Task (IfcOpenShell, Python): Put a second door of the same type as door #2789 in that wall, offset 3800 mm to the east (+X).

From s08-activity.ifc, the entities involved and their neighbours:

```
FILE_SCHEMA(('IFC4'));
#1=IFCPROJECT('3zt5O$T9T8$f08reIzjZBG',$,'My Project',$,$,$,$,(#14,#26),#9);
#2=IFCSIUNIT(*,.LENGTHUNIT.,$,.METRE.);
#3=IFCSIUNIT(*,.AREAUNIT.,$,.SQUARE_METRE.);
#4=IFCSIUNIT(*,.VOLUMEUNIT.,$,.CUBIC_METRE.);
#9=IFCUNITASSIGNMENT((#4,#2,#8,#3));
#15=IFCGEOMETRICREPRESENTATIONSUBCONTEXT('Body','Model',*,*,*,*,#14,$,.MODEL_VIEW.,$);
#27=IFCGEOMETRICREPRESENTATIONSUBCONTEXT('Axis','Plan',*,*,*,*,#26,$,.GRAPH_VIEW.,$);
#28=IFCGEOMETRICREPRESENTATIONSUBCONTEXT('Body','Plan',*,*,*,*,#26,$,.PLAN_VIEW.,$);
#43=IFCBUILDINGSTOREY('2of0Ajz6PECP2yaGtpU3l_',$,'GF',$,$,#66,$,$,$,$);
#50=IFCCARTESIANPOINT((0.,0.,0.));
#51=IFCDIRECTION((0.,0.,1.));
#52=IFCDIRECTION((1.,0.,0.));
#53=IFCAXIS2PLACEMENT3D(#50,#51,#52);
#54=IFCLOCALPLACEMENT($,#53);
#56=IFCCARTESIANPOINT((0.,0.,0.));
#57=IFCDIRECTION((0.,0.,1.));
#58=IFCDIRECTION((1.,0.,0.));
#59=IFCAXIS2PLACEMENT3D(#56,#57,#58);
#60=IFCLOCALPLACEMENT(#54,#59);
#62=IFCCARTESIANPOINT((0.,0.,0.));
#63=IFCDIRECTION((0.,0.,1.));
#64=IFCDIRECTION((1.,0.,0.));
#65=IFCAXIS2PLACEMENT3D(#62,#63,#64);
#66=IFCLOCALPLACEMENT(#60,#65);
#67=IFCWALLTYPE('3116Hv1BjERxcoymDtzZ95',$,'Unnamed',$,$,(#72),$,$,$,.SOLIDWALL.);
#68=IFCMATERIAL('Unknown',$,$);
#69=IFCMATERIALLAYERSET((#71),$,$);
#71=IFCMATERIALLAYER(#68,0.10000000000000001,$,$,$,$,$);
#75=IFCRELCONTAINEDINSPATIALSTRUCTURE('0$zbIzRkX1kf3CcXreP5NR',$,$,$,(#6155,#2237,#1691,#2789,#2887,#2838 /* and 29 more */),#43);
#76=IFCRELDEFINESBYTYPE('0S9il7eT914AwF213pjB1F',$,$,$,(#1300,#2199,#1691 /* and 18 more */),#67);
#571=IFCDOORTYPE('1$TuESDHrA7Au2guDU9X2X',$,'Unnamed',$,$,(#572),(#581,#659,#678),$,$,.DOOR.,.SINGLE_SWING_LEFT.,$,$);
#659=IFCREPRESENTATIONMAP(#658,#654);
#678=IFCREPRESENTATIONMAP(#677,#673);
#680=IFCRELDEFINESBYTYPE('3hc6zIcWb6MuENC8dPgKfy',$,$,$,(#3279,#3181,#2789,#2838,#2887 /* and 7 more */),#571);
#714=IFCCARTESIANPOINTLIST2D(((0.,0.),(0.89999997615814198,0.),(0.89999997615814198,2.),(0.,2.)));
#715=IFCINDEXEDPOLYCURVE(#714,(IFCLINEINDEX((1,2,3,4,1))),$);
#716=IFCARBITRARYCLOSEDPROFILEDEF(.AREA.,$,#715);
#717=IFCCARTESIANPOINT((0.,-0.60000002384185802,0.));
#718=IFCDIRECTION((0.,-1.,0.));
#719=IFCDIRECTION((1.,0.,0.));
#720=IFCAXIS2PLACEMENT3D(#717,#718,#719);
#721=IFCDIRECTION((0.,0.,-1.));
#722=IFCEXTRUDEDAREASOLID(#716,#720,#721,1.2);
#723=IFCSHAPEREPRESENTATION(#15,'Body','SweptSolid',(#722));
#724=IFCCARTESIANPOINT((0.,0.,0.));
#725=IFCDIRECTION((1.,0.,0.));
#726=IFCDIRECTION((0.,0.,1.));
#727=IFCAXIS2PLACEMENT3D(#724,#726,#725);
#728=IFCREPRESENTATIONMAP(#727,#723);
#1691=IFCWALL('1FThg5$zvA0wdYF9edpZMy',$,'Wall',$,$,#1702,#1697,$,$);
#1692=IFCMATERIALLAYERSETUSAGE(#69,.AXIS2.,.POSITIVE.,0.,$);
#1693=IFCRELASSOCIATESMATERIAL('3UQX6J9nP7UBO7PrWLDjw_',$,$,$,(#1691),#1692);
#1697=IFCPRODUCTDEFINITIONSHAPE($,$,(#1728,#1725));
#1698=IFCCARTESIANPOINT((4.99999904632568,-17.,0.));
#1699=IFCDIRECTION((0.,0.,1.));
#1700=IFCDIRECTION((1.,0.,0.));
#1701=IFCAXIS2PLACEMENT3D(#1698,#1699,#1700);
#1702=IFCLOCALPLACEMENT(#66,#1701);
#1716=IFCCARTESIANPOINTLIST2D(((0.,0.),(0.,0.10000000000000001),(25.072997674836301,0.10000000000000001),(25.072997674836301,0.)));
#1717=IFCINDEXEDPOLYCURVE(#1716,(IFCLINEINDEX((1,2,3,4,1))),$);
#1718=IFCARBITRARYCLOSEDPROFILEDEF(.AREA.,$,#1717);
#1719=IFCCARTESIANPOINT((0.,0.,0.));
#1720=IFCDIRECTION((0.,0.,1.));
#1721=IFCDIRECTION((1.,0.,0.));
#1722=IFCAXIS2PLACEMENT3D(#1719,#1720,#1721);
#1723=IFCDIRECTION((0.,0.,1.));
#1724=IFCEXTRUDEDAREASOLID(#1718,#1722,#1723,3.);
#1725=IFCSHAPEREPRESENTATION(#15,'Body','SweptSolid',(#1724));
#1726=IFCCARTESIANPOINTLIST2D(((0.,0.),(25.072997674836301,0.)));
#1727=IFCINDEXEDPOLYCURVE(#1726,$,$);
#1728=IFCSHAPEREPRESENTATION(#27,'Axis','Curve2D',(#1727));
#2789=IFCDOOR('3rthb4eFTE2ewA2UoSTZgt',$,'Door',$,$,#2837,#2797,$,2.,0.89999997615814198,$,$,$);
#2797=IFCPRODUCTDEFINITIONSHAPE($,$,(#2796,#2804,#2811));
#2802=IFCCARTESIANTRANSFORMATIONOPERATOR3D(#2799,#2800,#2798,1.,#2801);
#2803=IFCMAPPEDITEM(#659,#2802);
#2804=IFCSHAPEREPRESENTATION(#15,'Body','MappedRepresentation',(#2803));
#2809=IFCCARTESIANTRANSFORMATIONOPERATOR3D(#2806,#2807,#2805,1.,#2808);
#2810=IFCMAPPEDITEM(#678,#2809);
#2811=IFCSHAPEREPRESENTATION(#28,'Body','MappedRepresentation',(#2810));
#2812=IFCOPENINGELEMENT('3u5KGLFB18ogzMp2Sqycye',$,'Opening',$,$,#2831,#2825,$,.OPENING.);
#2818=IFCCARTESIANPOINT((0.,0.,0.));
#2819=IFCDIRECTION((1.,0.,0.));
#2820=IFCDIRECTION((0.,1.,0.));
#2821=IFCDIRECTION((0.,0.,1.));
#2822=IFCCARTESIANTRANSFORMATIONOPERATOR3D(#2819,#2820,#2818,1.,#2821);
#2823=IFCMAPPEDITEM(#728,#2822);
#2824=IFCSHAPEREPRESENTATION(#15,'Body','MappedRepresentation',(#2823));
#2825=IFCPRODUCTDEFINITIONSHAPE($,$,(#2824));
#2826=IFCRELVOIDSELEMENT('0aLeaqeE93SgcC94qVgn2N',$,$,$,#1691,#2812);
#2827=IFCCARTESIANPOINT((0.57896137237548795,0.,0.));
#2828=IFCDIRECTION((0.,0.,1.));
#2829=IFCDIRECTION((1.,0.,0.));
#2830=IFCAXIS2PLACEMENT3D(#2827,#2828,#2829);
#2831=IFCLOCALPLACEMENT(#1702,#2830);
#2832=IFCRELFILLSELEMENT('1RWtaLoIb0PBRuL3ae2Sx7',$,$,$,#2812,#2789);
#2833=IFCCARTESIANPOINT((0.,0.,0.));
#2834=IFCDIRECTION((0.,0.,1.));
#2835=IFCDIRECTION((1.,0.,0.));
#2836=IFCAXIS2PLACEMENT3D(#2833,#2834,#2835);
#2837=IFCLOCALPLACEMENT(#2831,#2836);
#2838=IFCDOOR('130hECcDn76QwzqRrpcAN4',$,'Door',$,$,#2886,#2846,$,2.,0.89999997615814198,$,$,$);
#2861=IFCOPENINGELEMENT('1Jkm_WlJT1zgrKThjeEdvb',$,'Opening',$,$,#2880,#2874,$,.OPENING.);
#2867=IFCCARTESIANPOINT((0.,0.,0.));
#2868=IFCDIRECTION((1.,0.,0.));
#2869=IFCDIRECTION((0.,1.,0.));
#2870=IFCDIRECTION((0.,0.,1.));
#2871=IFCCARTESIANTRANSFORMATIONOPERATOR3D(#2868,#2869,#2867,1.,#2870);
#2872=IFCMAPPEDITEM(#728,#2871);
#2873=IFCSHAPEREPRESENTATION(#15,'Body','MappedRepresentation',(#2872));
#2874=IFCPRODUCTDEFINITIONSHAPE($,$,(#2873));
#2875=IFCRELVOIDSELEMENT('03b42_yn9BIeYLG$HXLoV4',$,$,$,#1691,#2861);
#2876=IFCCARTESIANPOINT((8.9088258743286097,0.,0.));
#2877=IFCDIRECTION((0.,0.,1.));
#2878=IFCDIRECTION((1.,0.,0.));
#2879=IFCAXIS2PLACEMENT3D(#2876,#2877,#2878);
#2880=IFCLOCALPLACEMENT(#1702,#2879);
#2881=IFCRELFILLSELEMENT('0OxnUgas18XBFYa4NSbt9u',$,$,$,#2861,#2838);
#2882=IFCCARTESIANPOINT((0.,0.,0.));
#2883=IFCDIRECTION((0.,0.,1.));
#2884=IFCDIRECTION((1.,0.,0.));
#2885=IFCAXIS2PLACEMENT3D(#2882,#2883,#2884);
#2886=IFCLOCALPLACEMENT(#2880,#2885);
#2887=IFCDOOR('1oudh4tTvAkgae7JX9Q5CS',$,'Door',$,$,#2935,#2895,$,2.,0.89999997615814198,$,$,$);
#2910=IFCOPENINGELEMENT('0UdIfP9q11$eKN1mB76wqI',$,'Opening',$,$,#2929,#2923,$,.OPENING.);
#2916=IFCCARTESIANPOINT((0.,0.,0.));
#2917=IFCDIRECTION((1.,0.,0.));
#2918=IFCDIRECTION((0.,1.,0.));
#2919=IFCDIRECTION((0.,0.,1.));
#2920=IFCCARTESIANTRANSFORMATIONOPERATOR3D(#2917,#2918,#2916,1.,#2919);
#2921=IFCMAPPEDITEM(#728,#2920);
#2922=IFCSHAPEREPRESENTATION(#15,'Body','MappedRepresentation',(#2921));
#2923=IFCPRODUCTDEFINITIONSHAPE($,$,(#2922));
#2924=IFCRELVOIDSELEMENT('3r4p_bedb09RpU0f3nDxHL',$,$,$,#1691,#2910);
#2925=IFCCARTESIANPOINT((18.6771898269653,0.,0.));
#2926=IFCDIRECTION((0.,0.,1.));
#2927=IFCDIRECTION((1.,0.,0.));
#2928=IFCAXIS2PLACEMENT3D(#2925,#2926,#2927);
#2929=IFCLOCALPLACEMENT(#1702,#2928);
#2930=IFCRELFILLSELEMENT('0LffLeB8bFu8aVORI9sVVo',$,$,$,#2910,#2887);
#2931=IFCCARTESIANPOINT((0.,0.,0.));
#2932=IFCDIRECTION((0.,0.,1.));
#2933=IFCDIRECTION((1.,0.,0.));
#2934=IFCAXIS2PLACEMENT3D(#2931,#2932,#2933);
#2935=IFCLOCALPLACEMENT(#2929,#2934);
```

```python
import ifcopenshell
import ifcopenshell.api.feature
import ifcopenshell.api.geometry
import ifcopenshell.api.root
import ifcopenshell.geom
import ifcopenshell.util.element
import ifcopenshell.util.placement
import ifcopenshell.util.shape
import ifcopenshell.util.unit

model = ifcopenshell.open("s08-activity.ifc")
unit_scale = ifcopenshell.util.unit.calculate_unit_scale(model)
settings = ifcopenshell.geom.settings()


def volume(element):
    """Net volume in cubic metres, openings subtracted."""
    shape = ifcopenshell.geom.create_shape(settings, element)
    return ifcopenshell.util.shape.get_volume(shape.geometry)


door = model.by_id(2789)
opening = door.FillsVoids[0].RelatingOpeningElement
wall = opening.VoidsElements[0].RelatingBuildingElement
before = volume(wall)
shift = ifcopenshell.util.placement.get_local_placement(wall.ObjectPlacement)[:3, 0] * 3.8 / unit_scale

# copy_class copies the void relationship, type, container and properties, but no geometry.
new_opening = ifcopenshell.api.root.copy_class(model, product=opening)
new_opening.Representation = ifcopenshell.util.element.copy_deep(
    model, opening.Representation, exclude=["IfcGeometricRepresentationContext", "IfcRepresentationMap"]
)
new_door = ifcopenshell.api.root.copy_class(model, product=door)
new_door.Representation = ifcopenshell.util.element.copy_deep(
    model, door.Representation, exclude=["IfcGeometricRepresentationContext", "IfcRepresentationMap"]
)
ifcopenshell.api.feature.add_filling(model, opening=new_opening, element=new_door)

for old, new in ((opening, new_opening), (door, new_door)):
    matrix = ifcopenshell.util.placement.get_local_placement(old.ObjectPlacement)
    matrix[:3, 3] += shift
    ifcopenshell.api.geometry.edit_object_placement(model, product=new, matrix=matrix, is_si=False)

after = volume(wall)

print(f"wall volume {before:.3f} -> {after:.3f} m3")

model.write("s08-activity_updated.ifc")
```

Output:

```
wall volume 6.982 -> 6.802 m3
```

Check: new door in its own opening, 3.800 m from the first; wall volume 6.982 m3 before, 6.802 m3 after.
